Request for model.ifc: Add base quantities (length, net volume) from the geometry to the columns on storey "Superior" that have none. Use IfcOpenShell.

First a look at what the model holds.

```python
import ifcopenshell
import ifcopenshell.util.element
import ifcopenshell.util.unit

model = ifcopenshell.open("model.ifc")
print(model.schema)
for unit_type in ("LENGTHUNIT", "AREAUNIT", "VOLUMEUNIT"):
    print(unit_type, ifcopenshell.util.unit.calculate_unit_scale(model, unit_type))
storey = next(s for s in model.by_type("IfcBuildingStorey") if s.Name == "Superior")
columns = [e for e in ifcopenshell.util.element.get_decomposition(storey) if e.is_a("IfcColumn")]
for e in sorted(columns, key=lambda e: e.id()):
    print(e.id(), e.is_a(), e.Name, list(ifcopenshell.util.element.get_psets(e, qtos_only=True)), sep=" | ")
```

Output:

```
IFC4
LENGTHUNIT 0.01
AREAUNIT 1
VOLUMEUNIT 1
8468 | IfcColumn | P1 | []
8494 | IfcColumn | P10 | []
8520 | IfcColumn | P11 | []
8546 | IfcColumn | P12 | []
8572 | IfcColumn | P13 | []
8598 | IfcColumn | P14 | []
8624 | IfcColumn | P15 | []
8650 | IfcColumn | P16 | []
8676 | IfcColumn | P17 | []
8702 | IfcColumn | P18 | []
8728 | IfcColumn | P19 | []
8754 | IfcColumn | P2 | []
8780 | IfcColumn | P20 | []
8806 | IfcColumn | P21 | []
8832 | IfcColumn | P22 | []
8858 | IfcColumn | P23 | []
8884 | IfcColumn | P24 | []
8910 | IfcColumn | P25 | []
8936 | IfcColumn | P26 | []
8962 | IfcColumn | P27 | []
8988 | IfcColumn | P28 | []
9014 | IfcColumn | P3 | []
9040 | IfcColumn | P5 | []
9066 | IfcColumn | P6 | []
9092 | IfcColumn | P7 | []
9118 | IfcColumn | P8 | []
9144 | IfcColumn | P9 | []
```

```python
import ifcopenshell
import ifcopenshell.api.pset
import ifcopenshell.geom
import ifcopenshell.util.element
import ifcopenshell.util.shape
import ifcopenshell.util.unit

model = ifcopenshell.open("model.ifc")
unit_scale = ifcopenshell.util.unit.calculate_unit_scale(model)
volume_scale = ifcopenshell.util.unit.calculate_unit_scale(model, "VOLUMEUNIT")
settings = ifcopenshell.geom.settings()

storey = next(s for s in model.by_type("IfcBuildingStorey") if s.Name == "Superior")
columns = [e for e in ifcopenshell.util.element.get_decomposition(storey) if e.is_a("IfcColumn")]

for e in sorted(columns, key=lambda e: e.id()):
    if ifcopenshell.util.element.get_psets(e, qtos_only=True, should_inherit=False):
        continue
    # Geometry comes back in metres, in the element's own axes.
    shape = ifcopenshell.geom.create_shape(settings, e)
    values = {
        "Length": ifcopenshell.util.shape.get_z(shape.geometry) / unit_scale,
        "NetVolume": ifcopenshell.util.shape.get_volume(shape.geometry) / volume_scale,
    }
    qto = ifcopenshell.api.pset.add_qto(model, product=e, name="Qto_ColumnBaseQuantities")
    ifcopenshell.api.pset.edit_qto(model, qto=qto, properties=values)
    print(e.id(), {k: round(v, 3) for k, v in values.items()})

model.write("model_edited.ifc")
```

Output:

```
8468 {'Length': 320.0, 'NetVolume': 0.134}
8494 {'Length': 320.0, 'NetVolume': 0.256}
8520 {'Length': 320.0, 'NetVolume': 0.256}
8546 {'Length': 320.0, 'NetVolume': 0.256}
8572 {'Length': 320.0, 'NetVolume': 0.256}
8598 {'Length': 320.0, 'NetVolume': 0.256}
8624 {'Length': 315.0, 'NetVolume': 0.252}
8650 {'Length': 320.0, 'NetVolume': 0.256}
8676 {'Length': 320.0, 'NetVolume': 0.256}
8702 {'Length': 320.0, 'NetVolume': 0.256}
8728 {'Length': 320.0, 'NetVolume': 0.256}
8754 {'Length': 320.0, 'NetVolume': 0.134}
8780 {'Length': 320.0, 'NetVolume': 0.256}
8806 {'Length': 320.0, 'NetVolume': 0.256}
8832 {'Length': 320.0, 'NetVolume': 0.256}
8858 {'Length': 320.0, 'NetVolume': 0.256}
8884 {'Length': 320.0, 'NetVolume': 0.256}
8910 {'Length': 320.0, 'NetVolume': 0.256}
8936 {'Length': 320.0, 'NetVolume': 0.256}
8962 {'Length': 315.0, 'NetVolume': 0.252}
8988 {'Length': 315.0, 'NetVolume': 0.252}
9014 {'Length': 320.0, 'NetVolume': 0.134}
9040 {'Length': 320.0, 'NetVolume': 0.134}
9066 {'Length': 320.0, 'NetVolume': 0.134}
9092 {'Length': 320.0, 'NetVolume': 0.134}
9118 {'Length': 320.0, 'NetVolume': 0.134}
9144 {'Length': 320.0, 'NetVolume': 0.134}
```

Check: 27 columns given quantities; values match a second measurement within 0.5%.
